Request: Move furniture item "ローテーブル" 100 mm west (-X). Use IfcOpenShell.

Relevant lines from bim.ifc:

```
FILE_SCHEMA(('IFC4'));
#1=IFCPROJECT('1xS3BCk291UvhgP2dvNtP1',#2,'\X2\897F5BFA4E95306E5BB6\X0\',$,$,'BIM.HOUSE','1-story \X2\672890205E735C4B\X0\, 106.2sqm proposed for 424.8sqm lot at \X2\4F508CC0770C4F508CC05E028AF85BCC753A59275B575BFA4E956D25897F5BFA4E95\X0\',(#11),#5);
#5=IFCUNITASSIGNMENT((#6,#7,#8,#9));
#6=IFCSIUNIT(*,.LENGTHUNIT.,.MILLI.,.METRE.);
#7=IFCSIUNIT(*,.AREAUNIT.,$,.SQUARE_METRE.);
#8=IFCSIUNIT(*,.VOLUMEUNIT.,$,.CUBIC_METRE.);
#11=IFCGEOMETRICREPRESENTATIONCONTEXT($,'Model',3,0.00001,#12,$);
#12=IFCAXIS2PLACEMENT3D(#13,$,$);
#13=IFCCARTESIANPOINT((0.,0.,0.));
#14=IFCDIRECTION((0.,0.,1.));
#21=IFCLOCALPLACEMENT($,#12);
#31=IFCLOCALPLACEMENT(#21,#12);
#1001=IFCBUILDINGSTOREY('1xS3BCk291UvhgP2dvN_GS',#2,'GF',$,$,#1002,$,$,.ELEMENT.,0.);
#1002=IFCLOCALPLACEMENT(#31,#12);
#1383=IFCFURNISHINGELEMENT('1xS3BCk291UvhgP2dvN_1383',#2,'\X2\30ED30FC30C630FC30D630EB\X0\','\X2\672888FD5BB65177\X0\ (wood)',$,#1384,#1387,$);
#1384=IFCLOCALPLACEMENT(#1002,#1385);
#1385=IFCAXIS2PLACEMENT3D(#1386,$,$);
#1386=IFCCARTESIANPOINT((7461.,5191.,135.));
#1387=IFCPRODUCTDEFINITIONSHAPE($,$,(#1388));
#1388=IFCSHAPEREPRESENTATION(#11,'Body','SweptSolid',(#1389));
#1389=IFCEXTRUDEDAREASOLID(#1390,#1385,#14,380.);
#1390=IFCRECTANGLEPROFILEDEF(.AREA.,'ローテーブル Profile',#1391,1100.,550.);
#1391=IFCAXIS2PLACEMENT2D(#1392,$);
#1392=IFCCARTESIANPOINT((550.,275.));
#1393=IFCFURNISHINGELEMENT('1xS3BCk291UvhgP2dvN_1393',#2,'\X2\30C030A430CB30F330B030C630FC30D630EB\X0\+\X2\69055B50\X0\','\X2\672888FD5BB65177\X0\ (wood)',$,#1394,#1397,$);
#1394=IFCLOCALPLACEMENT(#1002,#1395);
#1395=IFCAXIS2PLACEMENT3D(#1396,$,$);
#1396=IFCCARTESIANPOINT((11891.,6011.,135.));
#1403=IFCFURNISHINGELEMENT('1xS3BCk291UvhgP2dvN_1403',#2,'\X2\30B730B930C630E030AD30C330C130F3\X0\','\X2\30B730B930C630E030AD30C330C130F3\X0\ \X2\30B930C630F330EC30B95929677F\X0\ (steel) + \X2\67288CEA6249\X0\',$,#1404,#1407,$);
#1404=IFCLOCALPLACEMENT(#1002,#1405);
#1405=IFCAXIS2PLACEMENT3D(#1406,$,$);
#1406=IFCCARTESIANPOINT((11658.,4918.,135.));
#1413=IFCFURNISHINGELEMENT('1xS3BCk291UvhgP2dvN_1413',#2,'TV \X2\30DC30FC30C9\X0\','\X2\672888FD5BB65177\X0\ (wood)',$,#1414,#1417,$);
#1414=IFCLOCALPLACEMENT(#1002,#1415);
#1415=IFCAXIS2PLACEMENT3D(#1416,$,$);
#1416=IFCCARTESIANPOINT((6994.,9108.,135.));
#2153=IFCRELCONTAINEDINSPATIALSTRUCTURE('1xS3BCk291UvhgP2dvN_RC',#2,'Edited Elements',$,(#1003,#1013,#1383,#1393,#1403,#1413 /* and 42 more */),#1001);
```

```python
import ifcopenshell
import ifcopenshell.api.geometry
import ifcopenshell.util.placement
import ifcopenshell.util.unit

model = ifcopenshell.open("bim.ifc")
unit_scale = ifcopenshell.util.unit.calculate_unit_scale(model)

item = model.by_guid("1xS3BCk291UvhgP2dvN_1383")
matrix = ifcopenshell.util.placement.get_local_placement(item.ObjectPlacement)
matrix[0, 3] -= 0.1 / unit_scale
ifcopenshell.api.geometry.edit_object_placement(model, product=item, matrix=matrix, is_si=False)

print(ifcopenshell.util.placement.get_local_placement(item.ObjectPlacement).round(3) + 0.0)

model.write("bim_v2.ifc")
```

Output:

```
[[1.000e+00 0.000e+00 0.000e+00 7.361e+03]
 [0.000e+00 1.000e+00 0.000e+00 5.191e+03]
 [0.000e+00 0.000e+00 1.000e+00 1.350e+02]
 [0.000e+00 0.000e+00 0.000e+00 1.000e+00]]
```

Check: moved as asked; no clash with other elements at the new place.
